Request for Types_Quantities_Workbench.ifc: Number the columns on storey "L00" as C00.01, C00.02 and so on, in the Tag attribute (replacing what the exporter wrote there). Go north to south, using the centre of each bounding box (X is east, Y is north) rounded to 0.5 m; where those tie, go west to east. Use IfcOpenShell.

First a look at what the model holds.

```python
import ifcopenshell
import ifcopenshell.util.element
import ifcopenshell.util.placement

model = ifcopenshell.open("Types_Quantities_Workbench.ifc")
print(model.schema)
storey = next(s for s in model.by_type("IfcBuildingStorey") if s.Name == "L00")
columns = [e for e in ifcopenshell.util.element.get_decomposition(storey) if e.is_a("IfcColumn")]
for e in sorted(columns, key=lambda e: e.id()):
    origin = ifcopenshell.util.placement.get_local_placement(e.ObjectPlacement)[:3, 3]
    print(e.id(), e.Tag, e.Name, origin.round(2) + 0.0, sep=" | ")
```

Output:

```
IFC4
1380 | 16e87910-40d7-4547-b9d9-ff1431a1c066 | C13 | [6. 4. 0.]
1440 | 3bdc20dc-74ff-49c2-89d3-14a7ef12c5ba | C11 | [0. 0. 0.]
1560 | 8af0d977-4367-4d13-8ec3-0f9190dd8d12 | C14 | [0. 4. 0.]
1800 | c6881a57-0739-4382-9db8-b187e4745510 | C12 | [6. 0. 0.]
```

```python
import ifcopenshell
import ifcopenshell.geom
import ifcopenshell.util.element
import ifcopenshell.util.shape

model = ifcopenshell.open("Types_Quantities_Workbench.ifc")
settings = ifcopenshell.geom.settings()
settings.set("use-world-coords", True)


def centre(element):
    shape = ifcopenshell.geom.create_shape(settings, element)
    return ifcopenshell.util.shape.get_bbox_centroid(shape.geometry)


storey = next(s for s in model.by_type("IfcBuildingStorey") if s.Name == "L00")
columns = [e for e in ifcopenshell.util.element.get_decomposition(storey) if e.is_a("IfcColumn")]

# Insertion points can sit at a corner or the storey origin, so sort by the geometry (in metres).
centres = {e: centre(e) for e in columns}
columns.sort(key=lambda e: (-round(centres[e][1] / 0.5), centres[e][0]))

for i, e in enumerate(columns, start=1):
    number = f"C00.{i:02d}"
    e.Tag = number
    print(e.id(), number)

model.write("Types_Quantities_Workbench-out.ifc")
```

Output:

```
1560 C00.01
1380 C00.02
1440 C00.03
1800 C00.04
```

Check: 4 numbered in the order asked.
